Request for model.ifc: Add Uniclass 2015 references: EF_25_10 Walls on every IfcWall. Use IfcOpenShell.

First a look at what the model holds.

```python
import ifcopenshell

model = ifcopenshell.open("model.ifc")
print(model.schema)
print("classifications:", [c.Name for c in model.by_type("IfcClassification")])
for ifc_class in ("IfcDoor", "IfcRoof", "IfcStair", "IfcWall", "IfcWindow"):
    print(ifc_class, len(model.by_type(ifc_class)))
```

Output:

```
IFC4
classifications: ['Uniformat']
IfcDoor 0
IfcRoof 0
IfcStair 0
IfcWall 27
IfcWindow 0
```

```python
import ifcopenshell
import ifcopenshell.api.classification

model = ifcopenshell.open("model.ifc")

system = ifcopenshell.api.classification.add_classification(model, classification="Uniclass 2015")

codes = {
    "IfcWall": ("EF_25_10", "Walls"),
}
for ifc_class, (code, name) in codes.items():
    products = model.by_type(ifc_class)
    ifcopenshell.api.classification.add_reference(
        model, products=products, classification=system, identification=code, name=name
    )
    print(code, len(products))

model.write("model_edited.ifc")
```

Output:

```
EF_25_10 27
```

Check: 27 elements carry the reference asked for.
